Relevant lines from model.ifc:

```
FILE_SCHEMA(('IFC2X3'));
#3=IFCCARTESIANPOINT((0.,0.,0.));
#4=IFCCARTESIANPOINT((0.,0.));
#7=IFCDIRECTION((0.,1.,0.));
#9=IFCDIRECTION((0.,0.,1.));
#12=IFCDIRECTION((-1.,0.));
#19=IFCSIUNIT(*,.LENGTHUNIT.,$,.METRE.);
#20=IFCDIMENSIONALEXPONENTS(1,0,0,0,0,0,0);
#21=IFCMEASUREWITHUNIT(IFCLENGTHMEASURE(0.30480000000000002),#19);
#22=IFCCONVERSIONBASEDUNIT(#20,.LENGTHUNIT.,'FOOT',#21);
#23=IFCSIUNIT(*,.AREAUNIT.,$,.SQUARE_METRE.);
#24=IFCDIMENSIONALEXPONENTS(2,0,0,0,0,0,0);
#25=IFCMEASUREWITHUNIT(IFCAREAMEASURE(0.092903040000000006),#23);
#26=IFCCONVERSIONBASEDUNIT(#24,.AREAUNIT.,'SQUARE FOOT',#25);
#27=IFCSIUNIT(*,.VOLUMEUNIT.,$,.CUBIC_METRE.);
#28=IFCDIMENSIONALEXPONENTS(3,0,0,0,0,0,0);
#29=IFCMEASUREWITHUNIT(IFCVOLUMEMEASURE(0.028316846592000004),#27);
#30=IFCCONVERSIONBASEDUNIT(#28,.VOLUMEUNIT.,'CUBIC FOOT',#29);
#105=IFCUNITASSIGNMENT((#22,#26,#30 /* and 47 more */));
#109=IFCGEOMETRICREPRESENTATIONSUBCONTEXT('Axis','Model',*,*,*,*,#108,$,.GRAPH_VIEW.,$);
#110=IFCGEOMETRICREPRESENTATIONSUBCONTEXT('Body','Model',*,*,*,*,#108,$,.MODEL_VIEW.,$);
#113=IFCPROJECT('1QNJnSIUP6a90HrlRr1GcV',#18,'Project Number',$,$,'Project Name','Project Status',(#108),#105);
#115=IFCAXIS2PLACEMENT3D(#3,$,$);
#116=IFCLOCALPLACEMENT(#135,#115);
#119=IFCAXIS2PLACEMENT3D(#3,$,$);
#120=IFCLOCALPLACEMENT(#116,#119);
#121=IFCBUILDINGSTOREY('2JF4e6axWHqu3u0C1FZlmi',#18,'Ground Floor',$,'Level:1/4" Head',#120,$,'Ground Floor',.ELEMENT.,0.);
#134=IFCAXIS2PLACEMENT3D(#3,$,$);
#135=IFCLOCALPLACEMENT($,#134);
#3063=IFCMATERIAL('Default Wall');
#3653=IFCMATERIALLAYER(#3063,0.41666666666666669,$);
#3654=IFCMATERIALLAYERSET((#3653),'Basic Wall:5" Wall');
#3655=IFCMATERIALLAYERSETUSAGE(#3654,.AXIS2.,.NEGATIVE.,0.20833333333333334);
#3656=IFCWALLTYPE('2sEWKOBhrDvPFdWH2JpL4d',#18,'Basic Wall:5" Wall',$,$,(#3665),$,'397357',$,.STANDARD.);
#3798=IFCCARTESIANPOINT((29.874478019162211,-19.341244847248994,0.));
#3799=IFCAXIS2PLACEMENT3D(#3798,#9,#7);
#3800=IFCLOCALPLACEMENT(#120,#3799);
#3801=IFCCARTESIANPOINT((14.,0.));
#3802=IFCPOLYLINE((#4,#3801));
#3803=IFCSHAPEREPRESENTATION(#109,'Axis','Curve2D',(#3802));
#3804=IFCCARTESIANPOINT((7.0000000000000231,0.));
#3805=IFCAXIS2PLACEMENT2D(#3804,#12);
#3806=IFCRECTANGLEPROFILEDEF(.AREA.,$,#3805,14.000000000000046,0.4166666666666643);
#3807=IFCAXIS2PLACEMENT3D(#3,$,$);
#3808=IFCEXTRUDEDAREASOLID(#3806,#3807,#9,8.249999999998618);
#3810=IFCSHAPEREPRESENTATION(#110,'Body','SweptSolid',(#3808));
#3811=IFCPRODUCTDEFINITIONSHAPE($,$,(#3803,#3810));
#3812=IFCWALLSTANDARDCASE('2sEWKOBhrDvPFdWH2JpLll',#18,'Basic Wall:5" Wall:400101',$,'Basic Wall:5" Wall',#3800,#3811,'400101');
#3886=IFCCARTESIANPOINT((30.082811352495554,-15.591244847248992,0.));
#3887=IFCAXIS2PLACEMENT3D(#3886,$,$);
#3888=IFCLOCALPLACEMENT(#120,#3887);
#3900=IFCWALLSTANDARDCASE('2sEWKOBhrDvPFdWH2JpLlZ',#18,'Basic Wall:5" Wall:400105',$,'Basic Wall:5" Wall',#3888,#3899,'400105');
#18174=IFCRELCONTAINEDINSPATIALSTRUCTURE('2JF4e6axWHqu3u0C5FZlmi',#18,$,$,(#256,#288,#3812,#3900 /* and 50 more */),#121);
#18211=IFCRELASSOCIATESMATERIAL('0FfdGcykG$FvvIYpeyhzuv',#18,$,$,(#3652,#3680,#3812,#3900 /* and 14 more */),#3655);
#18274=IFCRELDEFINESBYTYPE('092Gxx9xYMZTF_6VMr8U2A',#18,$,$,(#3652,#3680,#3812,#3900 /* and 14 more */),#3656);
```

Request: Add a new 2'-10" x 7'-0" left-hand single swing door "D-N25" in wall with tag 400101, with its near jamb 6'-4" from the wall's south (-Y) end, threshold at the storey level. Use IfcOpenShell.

```python
import numpy as np
import ifcopenshell
import ifcopenshell.api.feature
import ifcopenshell.api.geometry
import ifcopenshell.api.root
import ifcopenshell.api.spatial
import ifcopenshell.api.type
import ifcopenshell.geom
import ifcopenshell.util.element
import ifcopenshell.util.placement
import ifcopenshell.util.representation
import ifcopenshell.util.shape
import ifcopenshell.util.unit

model = ifcopenshell.open("model.ifc")
unit_scale = ifcopenshell.util.unit.calculate_unit_scale(model)
settings = ifcopenshell.geom.settings()


def volume(element):
    """Net volume in cubic metres, openings subtracted."""
    shape = ifcopenshell.geom.create_shape(settings, element)
    return ifcopenshell.util.shape.get_volume(shape.geometry)


wall = model.by_guid("2sEWKOBhrDvPFdWH2JpLll")
storey = ifcopenshell.util.element.get_container(wall, ifc_class="IfcBuildingStorey")
context = ifcopenshell.util.representation.get_context(model, "Model", "Body", "MODEL_VIEW")
before = volume(wall)

width, height, from_end, sill = 0.8636, 2.1336, 1.9304, 0.0  # metres

# The wall runs along its own X axis, and the end named is its -X end.
wall_shape = ifcopenshell.geom.create_shape(settings, wall)
x, y, z = ifcopenshell.util.shape.get_vertices(wall_shape.geometry).T
start = x.min() + from_end
face, thickness = float(y.min()), float(y.max() - y.min())
wall_matrix = ifcopenshell.util.placement.get_local_placement(wall.ObjectPlacement)
level = ifcopenshell.util.placement.get_local_placement(storey.ObjectPlacement)[2, 3]


def in_wall(x, y):
    """Placement at x, y metres in the wall's axes, at sill height."""
    matrix = wall_matrix.copy()
    matrix[:, 3] = wall_matrix @ np.array([x / unit_scale, y / unit_scale, 0.0, 1.0])
    matrix[2, 3] = level + sill / unit_scale
    return matrix


# Opening: a box that overshoots both wall faces by 50 mm.
opening = ifcopenshell.api.root.create_entity(model, ifc_class="IfcOpeningElement")
box = ifcopenshell.api.geometry.add_wall_representation(
    model, context=context, length=width, height=height, thickness=thickness + 0.1
)
ifcopenshell.api.geometry.assign_representation(model, product=opening, representation=box)
ifcopenshell.api.geometry.edit_object_placement(model, product=opening, matrix=in_wall(start, face - 0.05), is_si=False)
ifcopenshell.api.feature.add_feature(model, feature=opening, element=wall)

door = ifcopenshell.api.root.create_entity(model, ifc_class="IfcDoor", name="D-N25")
door.OverallWidth, door.OverallHeight = width / unit_scale, height / unit_scale
body = ifcopenshell.api.geometry.add_door_representation(
    model,
    context=context,
    overall_width=door.OverallWidth,
    overall_height=door.OverallHeight,
    operation_type="SINGLE_SWING_LEFT",
    lining_properties={"LiningDepth": thickness / unit_scale, "ThresholdDepth": thickness / unit_scale},
)
ifcopenshell.api.geometry.assign_representation(model, product=door, representation=body)
ifcopenshell.api.spatial.assign_container(model, products=[door], relating_structure=storey)
fills = ifcopenshell.api.feature.add_filling(model, opening=opening, element=door)
fills.OwnerHistory = door.OwnerHistory  # required in IFC2X3

# IFC2X3 keeps the operation on the door style.
style = ifcopenshell.api.root.create_entity(model, ifc_class="IfcDoorStyle", name="D-N25")
style.OperationType, style.ConstructionType = "SINGLE_SWING_LEFT", "NOTDEFINED"
style.ParameterTakesPrecedence = style.Sizeable = False
ifcopenshell.api.type.assign_type(model, related_objects=[door], relating_type=style)

# The lining spans the wall, so the door starts at the wall face.
ifcopenshell.api.geometry.edit_object_placement(model, product=door, matrix=in_wall(start, face), is_si=False)

after = volume(wall)

print(f"wall volume {before:.3f} -> {after:.3f} m3")

model.write("model_rev.ifc")
```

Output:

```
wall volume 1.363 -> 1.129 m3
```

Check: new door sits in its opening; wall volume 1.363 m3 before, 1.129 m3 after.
